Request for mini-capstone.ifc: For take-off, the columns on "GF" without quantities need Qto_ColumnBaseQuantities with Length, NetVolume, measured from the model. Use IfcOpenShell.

First a look at what the model holds.

```python
import ifcopenshell
import ifcopenshell.util.element
import ifcopenshell.util.unit

model = ifcopenshell.open("mini-capstone.ifc")
print(model.schema)
for unit_type in ("LENGTHUNIT", "AREAUNIT", "VOLUMEUNIT"):
    print(unit_type, ifcopenshell.util.unit.calculate_unit_scale(model, unit_type))
storey = next(s for s in model.by_type("IfcBuildingStorey") if s.Name == "GF")
columns = [e for e in ifcopenshell.util.element.get_decomposition(storey) if e.is_a("IfcColumn")]
for e in sorted(columns, key=lambda e: e.id()):
    print(e.id(), e.is_a(), e.Name, list(ifcopenshell.util.element.get_psets(e, qtos_only=True)), sep=" | ")
```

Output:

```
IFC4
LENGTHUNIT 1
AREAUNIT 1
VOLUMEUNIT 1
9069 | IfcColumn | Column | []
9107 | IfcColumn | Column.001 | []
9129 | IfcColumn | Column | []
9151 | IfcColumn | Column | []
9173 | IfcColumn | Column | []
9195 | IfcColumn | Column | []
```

```python
import ifcopenshell
import ifcopenshell.api.pset
import ifcopenshell.geom
import ifcopenshell.util.element
import ifcopenshell.util.shape
import ifcopenshell.util.unit

model = ifcopenshell.open("mini-capstone.ifc")
unit_scale = ifcopenshell.util.unit.calculate_unit_scale(model)
volume_scale = ifcopenshell.util.unit.calculate_unit_scale(model, "VOLUMEUNIT")
settings = ifcopenshell.geom.settings()

storey = next(s for s in model.by_type("IfcBuildingStorey") if s.Name == "GF")
columns = [e for e in ifcopenshell.util.element.get_decomposition(storey) if e.is_a("IfcColumn")]

for e in sorted(columns, key=lambda e: e.id()):
    if ifcopenshell.util.element.get_psets(e, qtos_only=True, should_inherit=False):
        continue
    # Geometry comes back in metres, in the element's own axes.
    shape = ifcopenshell.geom.create_shape(settings, e)
    values = {
        "Length": ifcopenshell.util.shape.get_z(shape.geometry) / unit_scale,
        "NetVolume": ifcopenshell.util.shape.get_volume(shape.geometry) / volume_scale,
    }
    qto = ifcopenshell.api.pset.add_qto(model, product=e, name="Qto_ColumnBaseQuantities")
    ifcopenshell.api.pset.edit_qto(model, qto=qto, properties=values)
    print(e.id(), {k: round(v, 3) for k, v in values.items()})

model.write("mini-capstone_edited.ifc")
```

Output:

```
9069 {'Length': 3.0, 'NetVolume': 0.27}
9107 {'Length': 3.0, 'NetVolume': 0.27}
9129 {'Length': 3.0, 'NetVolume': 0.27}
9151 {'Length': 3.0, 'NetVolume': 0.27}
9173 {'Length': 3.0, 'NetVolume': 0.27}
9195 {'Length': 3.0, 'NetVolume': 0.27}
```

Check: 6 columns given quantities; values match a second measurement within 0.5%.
